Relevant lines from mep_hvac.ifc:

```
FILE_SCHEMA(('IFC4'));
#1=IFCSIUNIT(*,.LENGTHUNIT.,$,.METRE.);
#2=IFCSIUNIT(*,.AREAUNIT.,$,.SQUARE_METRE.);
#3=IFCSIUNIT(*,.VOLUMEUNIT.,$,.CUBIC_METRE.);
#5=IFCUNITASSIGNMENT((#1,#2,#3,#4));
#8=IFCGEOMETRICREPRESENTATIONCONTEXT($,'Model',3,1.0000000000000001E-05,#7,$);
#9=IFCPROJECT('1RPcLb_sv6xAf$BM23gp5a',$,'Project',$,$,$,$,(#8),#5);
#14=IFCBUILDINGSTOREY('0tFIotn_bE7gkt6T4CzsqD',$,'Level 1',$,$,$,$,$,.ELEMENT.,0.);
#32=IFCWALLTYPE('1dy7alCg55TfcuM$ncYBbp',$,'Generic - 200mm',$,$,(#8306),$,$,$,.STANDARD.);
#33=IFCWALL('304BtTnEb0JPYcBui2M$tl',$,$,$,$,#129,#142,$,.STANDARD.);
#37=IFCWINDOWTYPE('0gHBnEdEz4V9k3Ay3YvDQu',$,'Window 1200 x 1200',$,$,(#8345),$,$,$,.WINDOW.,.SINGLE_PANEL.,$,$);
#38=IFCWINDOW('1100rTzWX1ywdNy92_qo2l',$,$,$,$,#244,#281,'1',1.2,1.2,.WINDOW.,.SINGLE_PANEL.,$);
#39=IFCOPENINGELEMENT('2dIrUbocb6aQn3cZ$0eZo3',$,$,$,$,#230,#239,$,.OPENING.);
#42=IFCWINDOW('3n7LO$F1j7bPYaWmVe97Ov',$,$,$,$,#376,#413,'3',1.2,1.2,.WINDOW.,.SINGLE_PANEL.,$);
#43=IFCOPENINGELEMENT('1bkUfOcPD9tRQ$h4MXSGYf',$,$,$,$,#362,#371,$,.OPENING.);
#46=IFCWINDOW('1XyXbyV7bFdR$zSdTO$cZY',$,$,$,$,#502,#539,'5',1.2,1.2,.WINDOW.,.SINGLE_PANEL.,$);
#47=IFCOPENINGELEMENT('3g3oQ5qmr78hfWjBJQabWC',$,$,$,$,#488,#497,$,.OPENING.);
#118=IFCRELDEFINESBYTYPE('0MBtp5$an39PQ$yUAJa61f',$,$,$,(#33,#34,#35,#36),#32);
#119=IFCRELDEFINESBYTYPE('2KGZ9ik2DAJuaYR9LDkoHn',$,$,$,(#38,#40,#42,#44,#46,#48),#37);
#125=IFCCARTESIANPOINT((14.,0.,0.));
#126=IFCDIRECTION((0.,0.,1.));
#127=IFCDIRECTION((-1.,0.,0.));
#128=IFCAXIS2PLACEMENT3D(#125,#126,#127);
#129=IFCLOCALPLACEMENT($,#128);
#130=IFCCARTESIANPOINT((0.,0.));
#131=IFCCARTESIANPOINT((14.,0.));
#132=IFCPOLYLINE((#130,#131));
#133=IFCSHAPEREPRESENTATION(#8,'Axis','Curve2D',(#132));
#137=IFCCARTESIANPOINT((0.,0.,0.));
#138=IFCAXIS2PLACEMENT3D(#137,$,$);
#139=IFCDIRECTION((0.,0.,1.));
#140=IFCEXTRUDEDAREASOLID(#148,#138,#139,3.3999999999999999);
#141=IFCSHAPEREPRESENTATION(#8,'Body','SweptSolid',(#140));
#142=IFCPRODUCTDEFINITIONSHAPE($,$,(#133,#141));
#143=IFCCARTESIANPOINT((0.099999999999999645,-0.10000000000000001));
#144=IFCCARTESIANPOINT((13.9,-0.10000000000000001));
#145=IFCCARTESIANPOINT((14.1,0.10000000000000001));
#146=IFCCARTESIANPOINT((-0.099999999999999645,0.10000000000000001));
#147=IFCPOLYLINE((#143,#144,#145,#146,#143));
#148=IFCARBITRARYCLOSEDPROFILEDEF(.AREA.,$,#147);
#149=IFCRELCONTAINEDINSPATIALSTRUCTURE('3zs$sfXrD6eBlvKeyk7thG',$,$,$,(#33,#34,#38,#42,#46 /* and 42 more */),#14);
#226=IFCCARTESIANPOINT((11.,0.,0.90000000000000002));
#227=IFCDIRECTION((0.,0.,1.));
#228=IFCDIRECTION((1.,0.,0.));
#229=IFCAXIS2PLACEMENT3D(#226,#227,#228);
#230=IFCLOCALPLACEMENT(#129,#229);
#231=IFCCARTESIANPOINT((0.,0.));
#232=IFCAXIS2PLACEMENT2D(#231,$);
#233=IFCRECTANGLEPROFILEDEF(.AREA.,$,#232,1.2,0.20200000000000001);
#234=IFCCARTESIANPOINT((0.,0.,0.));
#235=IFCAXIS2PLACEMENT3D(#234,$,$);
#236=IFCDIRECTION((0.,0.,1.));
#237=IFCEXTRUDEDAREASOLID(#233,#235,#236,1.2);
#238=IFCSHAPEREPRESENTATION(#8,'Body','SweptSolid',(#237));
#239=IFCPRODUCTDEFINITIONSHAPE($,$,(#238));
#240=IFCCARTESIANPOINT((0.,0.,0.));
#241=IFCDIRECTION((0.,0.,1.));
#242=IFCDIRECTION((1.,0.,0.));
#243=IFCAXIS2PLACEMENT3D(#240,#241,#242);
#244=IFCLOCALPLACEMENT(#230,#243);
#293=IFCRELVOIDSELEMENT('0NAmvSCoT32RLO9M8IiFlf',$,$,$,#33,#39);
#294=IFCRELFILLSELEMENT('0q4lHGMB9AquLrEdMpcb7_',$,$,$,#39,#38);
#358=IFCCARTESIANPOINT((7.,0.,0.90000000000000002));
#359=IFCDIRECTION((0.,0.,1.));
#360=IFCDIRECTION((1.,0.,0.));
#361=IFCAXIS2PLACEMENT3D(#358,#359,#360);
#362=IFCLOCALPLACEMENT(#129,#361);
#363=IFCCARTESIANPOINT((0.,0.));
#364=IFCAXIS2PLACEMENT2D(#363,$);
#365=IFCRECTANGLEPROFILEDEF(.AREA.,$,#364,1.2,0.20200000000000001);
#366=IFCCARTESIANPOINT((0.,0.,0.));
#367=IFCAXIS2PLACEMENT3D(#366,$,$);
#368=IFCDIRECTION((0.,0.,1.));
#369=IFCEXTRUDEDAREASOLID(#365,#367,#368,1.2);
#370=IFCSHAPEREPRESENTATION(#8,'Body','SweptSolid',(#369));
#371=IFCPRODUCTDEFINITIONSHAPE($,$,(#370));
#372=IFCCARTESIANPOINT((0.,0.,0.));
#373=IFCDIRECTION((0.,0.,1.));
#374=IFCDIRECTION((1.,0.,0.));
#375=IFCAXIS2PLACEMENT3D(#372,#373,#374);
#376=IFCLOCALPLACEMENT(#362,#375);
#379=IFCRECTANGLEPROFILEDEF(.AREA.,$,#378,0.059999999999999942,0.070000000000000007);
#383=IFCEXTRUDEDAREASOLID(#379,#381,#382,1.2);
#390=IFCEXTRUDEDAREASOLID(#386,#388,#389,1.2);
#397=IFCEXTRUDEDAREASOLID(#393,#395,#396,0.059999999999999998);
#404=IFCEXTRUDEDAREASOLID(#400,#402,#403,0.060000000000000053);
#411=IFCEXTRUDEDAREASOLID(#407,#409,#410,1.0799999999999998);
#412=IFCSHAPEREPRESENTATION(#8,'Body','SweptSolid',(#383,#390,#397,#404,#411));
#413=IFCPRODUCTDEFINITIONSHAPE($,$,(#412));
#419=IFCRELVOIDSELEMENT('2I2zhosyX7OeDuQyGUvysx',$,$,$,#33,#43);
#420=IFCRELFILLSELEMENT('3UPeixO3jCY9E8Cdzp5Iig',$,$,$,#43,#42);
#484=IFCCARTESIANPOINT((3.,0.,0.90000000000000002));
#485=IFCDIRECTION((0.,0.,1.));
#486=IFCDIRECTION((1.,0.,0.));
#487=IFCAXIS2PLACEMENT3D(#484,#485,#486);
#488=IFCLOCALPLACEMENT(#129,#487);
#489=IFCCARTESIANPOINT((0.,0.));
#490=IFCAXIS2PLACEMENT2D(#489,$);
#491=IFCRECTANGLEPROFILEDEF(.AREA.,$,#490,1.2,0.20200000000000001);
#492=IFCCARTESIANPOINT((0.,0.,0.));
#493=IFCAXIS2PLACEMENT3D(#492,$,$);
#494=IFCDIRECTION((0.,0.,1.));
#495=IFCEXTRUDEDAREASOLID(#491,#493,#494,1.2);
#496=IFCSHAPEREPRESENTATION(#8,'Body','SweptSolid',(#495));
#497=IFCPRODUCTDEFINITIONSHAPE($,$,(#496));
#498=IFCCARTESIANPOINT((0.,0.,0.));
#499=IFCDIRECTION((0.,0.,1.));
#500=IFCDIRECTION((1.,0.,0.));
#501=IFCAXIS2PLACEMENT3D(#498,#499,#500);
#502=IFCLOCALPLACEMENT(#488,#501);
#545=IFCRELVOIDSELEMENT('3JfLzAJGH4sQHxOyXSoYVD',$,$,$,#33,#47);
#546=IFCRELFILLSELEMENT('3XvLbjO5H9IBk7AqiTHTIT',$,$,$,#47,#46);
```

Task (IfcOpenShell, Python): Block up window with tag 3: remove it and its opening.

```python
import ifcopenshell
import ifcopenshell.api.feature
import ifcopenshell.api.root
import ifcopenshell.geom
import ifcopenshell.util.shape

model = ifcopenshell.open("mep_hvac.ifc")
settings = ifcopenshell.geom.settings()


def volume(element):
    """Net volume in cubic metres, openings subtracted."""
    shape = ifcopenshell.geom.create_shape(settings, element)
    return ifcopenshell.util.shape.get_volume(shape.geometry)


window = model.by_guid("3n7LO$F1j7bPYaWmVe97Ov")
opening = window.FillsVoids[0].RelatingOpeningElement
wall = opening.VoidsElements[0].RelatingBuildingElement
before = volume(wall)

ifcopenshell.api.root.remove_product(model, product=window)
ifcopenshell.api.feature.remove_feature(model, feature=opening)

after = volume(wall)

print(f"wall volume {before:.3f} -> {after:.3f} m3")

model.write("mep_hvac_rev.ifc")
```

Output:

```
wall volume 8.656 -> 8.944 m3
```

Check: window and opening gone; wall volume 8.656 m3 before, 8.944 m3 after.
